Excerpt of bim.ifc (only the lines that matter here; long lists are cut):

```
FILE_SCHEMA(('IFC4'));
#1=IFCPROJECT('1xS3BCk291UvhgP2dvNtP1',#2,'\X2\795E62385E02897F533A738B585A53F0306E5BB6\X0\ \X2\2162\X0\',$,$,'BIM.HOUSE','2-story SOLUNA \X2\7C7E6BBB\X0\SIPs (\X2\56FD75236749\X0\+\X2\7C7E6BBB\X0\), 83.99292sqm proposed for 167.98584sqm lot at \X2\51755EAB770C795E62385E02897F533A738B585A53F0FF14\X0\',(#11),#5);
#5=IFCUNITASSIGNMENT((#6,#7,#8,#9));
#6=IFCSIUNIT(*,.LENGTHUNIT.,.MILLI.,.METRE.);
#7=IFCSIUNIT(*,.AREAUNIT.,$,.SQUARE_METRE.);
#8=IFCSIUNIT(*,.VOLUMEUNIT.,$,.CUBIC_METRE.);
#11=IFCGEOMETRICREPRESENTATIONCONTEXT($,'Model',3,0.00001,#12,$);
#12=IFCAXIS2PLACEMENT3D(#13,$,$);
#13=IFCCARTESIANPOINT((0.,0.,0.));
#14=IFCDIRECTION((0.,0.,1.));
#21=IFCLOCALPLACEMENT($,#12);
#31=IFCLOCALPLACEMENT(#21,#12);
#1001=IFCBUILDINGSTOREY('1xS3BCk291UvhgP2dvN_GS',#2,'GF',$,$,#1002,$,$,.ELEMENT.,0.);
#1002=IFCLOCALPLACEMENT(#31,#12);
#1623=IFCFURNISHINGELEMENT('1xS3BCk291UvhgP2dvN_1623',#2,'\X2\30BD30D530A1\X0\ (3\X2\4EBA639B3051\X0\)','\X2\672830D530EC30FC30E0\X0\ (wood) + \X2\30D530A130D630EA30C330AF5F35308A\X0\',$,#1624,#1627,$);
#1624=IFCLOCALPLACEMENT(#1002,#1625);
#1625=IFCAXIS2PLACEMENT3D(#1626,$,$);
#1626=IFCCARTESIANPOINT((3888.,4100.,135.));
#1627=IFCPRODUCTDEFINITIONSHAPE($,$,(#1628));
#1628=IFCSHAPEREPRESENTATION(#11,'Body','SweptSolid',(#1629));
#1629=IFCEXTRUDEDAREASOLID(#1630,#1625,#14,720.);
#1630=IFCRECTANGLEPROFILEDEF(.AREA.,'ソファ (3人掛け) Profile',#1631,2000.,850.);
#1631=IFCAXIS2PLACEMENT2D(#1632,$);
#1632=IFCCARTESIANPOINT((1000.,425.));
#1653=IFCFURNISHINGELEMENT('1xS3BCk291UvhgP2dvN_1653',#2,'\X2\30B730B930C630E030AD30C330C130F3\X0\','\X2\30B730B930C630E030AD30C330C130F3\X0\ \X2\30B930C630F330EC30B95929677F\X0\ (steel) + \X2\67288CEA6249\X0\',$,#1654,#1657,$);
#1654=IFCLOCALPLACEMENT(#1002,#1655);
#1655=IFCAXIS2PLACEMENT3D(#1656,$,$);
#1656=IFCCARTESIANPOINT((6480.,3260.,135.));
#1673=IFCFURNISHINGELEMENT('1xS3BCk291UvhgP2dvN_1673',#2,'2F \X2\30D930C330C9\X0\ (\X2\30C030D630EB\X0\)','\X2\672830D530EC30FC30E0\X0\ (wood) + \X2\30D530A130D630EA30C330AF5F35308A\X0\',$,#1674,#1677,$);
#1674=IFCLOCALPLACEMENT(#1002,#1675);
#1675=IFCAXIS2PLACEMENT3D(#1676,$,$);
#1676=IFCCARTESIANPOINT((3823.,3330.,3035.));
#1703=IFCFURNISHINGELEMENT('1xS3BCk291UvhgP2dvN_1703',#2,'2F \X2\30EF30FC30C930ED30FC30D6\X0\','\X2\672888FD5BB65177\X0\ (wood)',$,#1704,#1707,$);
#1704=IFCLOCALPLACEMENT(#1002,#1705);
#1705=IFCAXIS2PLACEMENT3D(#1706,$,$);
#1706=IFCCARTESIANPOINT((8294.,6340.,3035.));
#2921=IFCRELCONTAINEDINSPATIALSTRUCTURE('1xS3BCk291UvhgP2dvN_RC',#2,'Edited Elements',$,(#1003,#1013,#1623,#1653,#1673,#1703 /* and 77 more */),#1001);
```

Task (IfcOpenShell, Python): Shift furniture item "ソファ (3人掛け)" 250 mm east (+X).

```python
import ifcopenshell
import ifcopenshell.api.geometry
import ifcopenshell.util.placement
import ifcopenshell.util.unit

model = ifcopenshell.open("bim.ifc")
unit_scale = ifcopenshell.util.unit.calculate_unit_scale(model)

item = model.by_guid("1xS3BCk291UvhgP2dvN_1623")
matrix = ifcopenshell.util.placement.get_local_placement(item.ObjectPlacement)
matrix[0, 3] += 0.25 / unit_scale
ifcopenshell.api.geometry.edit_object_placement(model, product=item, matrix=matrix, is_si=False)

print(ifcopenshell.util.placement.get_local_placement(item.ObjectPlacement).round(3) + 0.0)

model.write("bim_edited.ifc")
```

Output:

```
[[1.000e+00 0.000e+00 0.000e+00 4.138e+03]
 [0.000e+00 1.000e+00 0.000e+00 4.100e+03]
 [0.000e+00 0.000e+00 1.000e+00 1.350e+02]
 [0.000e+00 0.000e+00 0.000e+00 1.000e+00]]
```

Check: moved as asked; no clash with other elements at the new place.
